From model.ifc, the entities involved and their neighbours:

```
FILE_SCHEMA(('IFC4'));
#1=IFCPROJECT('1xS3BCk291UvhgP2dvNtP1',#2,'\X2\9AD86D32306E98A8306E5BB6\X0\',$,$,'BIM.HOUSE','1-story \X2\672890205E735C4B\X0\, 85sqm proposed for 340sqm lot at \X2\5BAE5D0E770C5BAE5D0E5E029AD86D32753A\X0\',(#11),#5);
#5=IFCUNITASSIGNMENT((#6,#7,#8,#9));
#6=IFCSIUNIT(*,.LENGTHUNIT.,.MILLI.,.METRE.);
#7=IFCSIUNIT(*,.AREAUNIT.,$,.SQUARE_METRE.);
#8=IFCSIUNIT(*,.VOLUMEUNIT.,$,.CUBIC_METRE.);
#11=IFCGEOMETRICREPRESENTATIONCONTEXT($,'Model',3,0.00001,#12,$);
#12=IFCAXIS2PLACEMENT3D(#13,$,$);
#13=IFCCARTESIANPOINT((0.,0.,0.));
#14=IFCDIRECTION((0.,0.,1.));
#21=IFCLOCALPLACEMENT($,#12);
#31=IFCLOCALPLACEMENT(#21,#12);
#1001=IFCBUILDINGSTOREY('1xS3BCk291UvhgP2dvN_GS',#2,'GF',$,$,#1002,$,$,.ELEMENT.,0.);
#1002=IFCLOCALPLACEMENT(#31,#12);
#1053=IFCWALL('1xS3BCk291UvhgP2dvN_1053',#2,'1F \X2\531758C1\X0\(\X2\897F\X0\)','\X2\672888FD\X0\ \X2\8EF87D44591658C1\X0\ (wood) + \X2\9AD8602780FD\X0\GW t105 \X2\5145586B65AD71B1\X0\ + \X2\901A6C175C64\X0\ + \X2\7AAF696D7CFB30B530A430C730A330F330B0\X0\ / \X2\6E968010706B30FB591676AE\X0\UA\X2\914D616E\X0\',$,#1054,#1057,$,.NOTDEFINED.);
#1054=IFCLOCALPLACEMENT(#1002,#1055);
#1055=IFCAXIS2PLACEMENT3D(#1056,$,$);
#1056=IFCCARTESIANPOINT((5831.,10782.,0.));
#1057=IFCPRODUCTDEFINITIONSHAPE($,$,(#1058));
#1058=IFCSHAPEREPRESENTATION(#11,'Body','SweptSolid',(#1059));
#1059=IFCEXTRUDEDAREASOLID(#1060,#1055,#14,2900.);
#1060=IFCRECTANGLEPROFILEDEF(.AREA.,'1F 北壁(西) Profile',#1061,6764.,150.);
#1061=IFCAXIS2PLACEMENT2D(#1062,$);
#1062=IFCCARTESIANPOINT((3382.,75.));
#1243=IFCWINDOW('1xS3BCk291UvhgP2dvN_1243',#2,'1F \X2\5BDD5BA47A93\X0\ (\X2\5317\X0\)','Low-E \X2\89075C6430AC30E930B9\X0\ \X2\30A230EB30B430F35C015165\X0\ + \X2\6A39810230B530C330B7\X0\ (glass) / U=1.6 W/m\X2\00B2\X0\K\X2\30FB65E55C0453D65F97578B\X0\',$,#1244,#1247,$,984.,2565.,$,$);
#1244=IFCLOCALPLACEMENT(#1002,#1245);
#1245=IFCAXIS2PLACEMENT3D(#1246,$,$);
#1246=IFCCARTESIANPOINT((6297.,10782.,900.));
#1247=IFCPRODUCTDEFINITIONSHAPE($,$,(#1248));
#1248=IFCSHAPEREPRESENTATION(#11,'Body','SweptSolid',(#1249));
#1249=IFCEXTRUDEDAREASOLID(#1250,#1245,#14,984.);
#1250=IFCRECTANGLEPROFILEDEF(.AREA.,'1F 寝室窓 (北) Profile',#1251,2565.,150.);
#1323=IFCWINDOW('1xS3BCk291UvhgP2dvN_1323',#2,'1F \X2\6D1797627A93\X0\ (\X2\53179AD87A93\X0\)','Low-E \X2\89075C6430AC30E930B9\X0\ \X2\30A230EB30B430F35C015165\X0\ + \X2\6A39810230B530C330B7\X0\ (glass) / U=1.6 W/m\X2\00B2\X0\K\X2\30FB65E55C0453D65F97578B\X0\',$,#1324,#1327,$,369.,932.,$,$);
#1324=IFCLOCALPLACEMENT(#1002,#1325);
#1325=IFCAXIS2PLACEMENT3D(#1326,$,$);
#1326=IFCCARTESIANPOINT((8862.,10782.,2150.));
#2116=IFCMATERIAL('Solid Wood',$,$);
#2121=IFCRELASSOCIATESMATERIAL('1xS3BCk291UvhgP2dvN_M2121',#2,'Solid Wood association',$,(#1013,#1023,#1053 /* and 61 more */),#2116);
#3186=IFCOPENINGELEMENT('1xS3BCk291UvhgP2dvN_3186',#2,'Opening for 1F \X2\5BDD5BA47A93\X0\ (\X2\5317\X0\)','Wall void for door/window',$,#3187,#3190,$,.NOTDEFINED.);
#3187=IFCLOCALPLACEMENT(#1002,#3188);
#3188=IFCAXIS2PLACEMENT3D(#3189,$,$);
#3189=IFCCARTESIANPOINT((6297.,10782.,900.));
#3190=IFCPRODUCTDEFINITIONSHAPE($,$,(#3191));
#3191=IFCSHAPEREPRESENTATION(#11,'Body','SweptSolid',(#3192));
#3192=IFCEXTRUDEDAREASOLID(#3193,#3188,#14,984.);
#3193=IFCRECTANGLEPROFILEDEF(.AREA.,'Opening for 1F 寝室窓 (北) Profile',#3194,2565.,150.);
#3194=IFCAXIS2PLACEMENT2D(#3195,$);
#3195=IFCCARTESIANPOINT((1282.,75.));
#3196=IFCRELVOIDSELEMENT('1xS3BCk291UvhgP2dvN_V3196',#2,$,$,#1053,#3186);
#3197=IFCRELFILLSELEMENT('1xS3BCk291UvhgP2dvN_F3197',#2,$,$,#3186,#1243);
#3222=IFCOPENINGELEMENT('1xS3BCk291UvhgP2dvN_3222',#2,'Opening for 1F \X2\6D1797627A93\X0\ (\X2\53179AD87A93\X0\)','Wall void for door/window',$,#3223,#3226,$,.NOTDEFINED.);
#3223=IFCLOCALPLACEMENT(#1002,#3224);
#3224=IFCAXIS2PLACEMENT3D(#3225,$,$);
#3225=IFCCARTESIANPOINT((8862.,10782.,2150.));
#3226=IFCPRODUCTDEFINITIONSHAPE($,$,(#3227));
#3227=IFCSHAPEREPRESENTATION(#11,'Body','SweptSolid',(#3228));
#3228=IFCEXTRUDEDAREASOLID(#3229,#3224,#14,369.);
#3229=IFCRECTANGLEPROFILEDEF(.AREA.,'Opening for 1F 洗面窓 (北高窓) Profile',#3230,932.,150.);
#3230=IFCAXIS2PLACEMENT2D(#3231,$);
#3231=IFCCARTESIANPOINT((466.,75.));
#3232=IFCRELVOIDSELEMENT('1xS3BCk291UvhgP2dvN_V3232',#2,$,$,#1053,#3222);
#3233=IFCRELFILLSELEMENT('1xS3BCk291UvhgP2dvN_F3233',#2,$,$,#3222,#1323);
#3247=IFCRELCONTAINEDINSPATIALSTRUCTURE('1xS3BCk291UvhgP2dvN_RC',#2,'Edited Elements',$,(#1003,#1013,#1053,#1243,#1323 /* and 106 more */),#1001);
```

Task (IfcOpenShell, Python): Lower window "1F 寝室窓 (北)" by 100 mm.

```python
import numpy as np
import ifcopenshell
import ifcopenshell.api.geometry
import ifcopenshell.util.placement
import ifcopenshell.util.unit

model = ifcopenshell.open("model.ifc")
unit_scale = ifcopenshell.util.unit.calculate_unit_scale(model)

window = model.by_id(1243)
opening = window.FillsVoids[0].RelatingOpeningElement
dz = -0.1 / unit_scale

shift = np.array([0.0, 0.0, dz])
# The window is not placed relative to its opening, so move both.
for product in (opening, window):
    matrix = ifcopenshell.util.placement.get_local_placement(product.ObjectPlacement)
    matrix[:3, 3] += shift
    ifcopenshell.api.geometry.edit_object_placement(model, product=product, matrix=matrix, is_si=False)

print(f"moved by {dz * unit_scale:+.3f} m")

model.write("model-out.ifc")
```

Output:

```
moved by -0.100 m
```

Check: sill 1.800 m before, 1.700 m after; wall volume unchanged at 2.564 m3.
